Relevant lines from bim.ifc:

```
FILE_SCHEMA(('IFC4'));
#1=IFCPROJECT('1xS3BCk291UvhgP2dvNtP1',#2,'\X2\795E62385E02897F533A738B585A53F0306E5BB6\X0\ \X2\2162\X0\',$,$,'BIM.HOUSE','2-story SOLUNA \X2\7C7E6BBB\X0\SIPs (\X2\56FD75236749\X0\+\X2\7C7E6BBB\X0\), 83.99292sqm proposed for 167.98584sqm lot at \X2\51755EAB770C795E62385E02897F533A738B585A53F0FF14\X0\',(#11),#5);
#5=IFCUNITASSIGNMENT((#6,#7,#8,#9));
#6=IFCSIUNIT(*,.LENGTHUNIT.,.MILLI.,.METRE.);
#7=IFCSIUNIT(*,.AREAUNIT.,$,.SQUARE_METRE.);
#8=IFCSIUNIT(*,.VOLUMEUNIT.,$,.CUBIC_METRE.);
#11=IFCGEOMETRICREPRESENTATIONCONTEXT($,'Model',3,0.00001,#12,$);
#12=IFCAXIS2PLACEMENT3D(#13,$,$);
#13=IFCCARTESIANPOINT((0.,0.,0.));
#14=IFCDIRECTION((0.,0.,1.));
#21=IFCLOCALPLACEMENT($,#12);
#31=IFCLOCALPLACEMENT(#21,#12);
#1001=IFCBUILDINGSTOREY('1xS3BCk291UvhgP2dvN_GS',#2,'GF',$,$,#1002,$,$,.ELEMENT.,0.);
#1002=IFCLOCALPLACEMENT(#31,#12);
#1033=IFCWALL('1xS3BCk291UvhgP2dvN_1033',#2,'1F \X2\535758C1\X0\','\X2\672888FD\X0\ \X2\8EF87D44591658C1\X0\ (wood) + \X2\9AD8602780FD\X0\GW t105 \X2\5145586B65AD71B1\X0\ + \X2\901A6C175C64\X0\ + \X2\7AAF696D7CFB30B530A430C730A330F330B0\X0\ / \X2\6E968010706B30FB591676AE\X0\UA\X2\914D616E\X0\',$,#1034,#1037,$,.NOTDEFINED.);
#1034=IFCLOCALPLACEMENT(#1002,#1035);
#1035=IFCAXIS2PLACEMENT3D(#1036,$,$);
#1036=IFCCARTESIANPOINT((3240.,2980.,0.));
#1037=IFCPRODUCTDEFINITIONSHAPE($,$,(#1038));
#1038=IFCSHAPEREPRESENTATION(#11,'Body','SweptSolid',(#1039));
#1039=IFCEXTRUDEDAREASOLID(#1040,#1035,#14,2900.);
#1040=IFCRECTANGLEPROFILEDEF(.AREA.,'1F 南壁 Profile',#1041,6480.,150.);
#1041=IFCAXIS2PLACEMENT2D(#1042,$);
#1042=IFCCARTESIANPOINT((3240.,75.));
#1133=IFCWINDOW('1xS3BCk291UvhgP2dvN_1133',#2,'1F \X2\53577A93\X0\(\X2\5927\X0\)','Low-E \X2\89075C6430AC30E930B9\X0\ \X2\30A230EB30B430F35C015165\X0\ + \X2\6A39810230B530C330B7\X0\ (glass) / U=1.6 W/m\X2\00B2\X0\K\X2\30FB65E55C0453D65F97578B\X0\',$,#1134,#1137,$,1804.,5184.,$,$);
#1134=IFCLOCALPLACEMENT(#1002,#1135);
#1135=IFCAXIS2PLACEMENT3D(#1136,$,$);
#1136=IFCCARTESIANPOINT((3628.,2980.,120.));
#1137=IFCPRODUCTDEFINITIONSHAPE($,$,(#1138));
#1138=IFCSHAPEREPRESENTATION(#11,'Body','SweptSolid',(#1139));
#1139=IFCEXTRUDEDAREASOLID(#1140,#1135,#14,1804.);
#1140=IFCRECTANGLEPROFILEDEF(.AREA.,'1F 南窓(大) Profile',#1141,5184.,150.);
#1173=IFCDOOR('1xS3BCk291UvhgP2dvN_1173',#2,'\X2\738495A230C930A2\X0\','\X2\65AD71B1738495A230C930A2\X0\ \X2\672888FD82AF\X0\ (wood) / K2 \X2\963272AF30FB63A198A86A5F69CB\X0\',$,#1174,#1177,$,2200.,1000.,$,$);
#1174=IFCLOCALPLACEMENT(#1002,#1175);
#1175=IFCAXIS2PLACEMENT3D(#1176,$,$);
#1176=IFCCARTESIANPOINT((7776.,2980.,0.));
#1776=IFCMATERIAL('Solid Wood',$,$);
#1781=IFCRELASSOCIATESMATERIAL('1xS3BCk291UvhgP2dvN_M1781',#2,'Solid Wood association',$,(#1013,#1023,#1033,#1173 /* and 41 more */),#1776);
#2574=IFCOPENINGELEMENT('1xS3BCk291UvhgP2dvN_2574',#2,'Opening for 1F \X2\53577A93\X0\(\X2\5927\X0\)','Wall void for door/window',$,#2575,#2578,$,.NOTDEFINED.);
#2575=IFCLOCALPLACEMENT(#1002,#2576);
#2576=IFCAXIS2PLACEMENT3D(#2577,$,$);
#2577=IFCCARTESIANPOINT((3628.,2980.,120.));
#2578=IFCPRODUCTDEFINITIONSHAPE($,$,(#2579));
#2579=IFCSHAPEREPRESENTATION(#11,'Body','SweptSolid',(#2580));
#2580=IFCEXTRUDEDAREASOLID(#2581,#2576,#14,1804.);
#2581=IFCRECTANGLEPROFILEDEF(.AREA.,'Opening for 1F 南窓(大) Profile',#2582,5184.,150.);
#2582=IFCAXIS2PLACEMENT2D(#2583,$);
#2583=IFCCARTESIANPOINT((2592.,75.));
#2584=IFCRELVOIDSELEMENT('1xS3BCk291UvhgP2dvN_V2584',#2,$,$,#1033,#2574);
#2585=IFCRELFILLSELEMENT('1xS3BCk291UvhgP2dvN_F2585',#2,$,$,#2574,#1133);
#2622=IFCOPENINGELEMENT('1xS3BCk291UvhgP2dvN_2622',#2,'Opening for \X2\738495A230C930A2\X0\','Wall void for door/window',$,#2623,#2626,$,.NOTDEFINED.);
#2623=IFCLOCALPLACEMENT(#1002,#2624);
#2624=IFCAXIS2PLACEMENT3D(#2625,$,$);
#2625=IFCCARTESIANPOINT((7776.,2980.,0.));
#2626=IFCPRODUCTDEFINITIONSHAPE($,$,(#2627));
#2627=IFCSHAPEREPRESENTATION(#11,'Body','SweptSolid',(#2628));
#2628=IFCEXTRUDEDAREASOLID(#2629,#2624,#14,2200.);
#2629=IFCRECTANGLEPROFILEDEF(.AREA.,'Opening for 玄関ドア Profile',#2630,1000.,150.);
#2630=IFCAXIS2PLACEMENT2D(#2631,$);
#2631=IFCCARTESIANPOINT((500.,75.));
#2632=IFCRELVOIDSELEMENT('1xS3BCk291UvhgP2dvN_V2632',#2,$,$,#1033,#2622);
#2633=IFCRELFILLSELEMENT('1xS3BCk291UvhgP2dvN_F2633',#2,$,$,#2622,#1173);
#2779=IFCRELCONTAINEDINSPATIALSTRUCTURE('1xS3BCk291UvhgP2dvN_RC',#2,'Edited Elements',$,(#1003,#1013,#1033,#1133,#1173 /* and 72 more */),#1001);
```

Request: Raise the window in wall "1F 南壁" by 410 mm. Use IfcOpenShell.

```python
import numpy as np
import ifcopenshell
import ifcopenshell.api.geometry
import ifcopenshell.util.placement
import ifcopenshell.util.unit

model = ifcopenshell.open("bim.ifc")
unit_scale = ifcopenshell.util.unit.calculate_unit_scale(model)

window = model.by_guid("1xS3BCk291UvhgP2dvN_1133")
opening = window.FillsVoids[0].RelatingOpeningElement
dz = 0.41 / unit_scale

shift = np.array([0.0, 0.0, dz])
# The window is not placed relative to its opening, so move both.
for product in (opening, window):
    matrix = ifcopenshell.util.placement.get_local_placement(product.ObjectPlacement)
    matrix[:3, 3] += shift
    ifcopenshell.api.geometry.edit_object_placement(model, product=product, matrix=matrix, is_si=False)

print(f"moved by {dz * unit_scale:+.3f} m")

model.write("bim_updated.ifc")
```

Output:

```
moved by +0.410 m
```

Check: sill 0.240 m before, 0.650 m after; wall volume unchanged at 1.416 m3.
